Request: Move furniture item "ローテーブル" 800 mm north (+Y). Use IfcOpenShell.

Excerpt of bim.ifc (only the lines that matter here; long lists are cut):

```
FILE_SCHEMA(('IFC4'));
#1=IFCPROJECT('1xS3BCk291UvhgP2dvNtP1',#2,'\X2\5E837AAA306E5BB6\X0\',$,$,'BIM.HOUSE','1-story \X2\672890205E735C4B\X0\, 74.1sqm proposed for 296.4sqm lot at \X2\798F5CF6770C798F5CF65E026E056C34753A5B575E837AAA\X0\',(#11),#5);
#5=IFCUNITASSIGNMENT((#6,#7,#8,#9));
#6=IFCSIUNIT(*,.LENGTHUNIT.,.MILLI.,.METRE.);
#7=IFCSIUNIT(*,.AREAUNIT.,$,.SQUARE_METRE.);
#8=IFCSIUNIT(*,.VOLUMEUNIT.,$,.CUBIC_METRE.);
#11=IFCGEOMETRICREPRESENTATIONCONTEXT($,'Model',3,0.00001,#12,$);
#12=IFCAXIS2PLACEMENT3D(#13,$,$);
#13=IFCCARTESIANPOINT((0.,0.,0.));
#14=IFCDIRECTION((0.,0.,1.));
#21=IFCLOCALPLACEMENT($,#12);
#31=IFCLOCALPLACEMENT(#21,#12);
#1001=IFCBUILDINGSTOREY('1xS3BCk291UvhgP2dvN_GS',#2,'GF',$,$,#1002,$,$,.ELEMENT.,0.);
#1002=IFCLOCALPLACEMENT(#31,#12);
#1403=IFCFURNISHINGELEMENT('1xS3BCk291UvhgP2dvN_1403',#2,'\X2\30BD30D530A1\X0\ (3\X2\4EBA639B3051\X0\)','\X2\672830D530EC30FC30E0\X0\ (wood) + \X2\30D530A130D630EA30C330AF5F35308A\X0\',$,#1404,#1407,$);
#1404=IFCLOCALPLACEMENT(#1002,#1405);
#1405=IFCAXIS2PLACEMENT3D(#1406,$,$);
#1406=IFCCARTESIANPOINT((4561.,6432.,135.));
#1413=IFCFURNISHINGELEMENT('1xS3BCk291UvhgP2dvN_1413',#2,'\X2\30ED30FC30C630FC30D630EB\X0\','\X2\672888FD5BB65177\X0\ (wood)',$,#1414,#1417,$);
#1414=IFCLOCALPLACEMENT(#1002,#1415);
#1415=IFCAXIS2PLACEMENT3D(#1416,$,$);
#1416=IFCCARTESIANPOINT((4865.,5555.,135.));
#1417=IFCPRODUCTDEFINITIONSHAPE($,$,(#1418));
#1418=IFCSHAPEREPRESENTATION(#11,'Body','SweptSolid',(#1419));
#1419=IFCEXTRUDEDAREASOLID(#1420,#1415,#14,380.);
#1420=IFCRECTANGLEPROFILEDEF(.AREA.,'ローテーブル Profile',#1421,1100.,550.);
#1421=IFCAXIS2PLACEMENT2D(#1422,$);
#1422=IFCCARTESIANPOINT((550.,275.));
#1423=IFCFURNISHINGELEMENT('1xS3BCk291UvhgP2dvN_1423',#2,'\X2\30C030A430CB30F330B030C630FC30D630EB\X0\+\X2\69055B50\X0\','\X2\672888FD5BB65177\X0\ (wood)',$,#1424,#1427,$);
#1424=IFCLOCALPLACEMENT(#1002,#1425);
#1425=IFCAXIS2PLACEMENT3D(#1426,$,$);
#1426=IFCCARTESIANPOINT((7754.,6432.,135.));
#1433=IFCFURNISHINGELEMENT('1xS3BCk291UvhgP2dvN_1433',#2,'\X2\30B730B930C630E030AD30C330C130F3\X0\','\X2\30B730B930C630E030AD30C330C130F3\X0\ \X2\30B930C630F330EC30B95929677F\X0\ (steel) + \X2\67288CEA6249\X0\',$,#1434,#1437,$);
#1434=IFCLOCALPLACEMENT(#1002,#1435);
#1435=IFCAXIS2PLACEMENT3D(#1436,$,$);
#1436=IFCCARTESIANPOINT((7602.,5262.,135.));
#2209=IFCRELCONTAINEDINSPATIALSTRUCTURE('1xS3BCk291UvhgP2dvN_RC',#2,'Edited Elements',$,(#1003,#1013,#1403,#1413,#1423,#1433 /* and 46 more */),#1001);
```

```python
import ifcopenshell
import ifcopenshell.api.geometry
import ifcopenshell.util.placement

model = ifcopenshell.open("bim.ifc")

item = model.by_id(1413)
matrix = ifcopenshell.util.placement.get_local_placement(item.ObjectPlacement)
matrix[1, 3] += 800.0
ifcopenshell.api.geometry.edit_object_placement(model, product=item, matrix=matrix, is_si=False)

print(ifcopenshell.util.placement.get_local_placement(item.ObjectPlacement).round(3) + 0.0)

model.write("bim-out.ifc")
```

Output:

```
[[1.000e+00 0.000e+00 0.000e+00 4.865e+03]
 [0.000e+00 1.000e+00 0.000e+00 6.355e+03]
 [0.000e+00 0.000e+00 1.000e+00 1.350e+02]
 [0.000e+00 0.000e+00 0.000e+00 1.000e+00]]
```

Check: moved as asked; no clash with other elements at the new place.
